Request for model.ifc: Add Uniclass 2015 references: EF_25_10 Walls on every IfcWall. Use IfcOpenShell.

First a look at what the model holds.

```python
import ifcopenshell

model = ifcopenshell.open("model.ifc")
print(model.schema)
print("classifications:", [c.Name for c in model.by_type("IfcClassification")])
for ifc_class in ("IfcDoor", "IfcRoof", "IfcStair", "IfcWall", "IfcWindow"):
    print(ifc_class, len(model.by_type(ifc_class)))
```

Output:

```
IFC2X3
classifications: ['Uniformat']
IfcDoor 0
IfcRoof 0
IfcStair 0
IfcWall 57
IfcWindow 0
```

```python
import ifcopenshell
import ifcopenshell.api.classification

model = ifcopenshell.open("model.ifc")

# IFC2X3 requires Source and Edition and has no link from the project to the system.
system = model.create_entity("IfcClassification", Source="NBS", Edition="2015", Name="Uniclass 2015")

codes = {
    "IfcWall": ("EF_25_10", "Walls"),
}
for ifc_class, (code, name) in codes.items():
    products = model.by_type(ifc_class)
    ifcopenshell.api.classification.add_reference(
        model, products=products, classification=system, identification=code, name=name
    )
    print(code, len(products))

model.write("model_v2.ifc")
```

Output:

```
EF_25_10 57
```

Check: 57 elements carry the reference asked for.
